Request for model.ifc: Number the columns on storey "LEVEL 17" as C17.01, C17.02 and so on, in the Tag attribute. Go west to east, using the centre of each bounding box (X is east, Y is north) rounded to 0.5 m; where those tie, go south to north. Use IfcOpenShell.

First a look at what the model holds.

```python
import ifcopenshell
import ifcopenshell.util.element
import ifcopenshell.util.placement

model = ifcopenshell.open("model.ifc")
print(model.schema)
storey = next(s for s in model.by_type("IfcBuildingStorey") if s.Name == "LEVEL 17")
columns = [e for e in ifcopenshell.util.element.get_decomposition(storey) if e.is_a("IfcColumn")]
for e in sorted(columns, key=lambda e: e.id()):
    origin = ifcopenshell.util.placement.get_local_placement(e.ObjectPlacement)[:3, 3]
    print(e.id(), e.Tag, e.Name, origin.round(2) + 0.0, sep=" | ")
```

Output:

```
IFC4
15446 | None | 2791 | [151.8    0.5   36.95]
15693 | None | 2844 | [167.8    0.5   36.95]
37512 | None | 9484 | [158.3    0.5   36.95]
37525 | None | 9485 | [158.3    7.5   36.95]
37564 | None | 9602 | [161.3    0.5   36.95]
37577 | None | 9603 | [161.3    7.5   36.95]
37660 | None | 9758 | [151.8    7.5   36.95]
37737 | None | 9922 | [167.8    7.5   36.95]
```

```python
import ifcopenshell
import ifcopenshell.geom
import ifcopenshell.util.element
import ifcopenshell.util.shape

model = ifcopenshell.open("model.ifc")
settings = ifcopenshell.geom.settings()
settings.set("use-world-coords", True)


def centre(element):
    shape = ifcopenshell.geom.create_shape(settings, element)
    return ifcopenshell.util.shape.get_bbox_centroid(shape.geometry)


storey = next(s for s in model.by_type("IfcBuildingStorey") if s.Name == "LEVEL 17")
columns = [e for e in ifcopenshell.util.element.get_decomposition(storey) if e.is_a("IfcColumn")]

# Insertion points can sit at a corner or the storey origin, so sort by the geometry (in metres).
centres = {e: centre(e) for e in columns}
columns.sort(key=lambda e: (round(centres[e][0] / 0.5), centres[e][1]))

for i, e in enumerate(columns, start=1):
    number = f"C17.{i:02d}"
    e.Tag = number
    print(e.id(), number)

model.write("model_edited.ifc")
```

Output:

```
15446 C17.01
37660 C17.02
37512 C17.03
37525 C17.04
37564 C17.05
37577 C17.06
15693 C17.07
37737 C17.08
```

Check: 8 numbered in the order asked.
